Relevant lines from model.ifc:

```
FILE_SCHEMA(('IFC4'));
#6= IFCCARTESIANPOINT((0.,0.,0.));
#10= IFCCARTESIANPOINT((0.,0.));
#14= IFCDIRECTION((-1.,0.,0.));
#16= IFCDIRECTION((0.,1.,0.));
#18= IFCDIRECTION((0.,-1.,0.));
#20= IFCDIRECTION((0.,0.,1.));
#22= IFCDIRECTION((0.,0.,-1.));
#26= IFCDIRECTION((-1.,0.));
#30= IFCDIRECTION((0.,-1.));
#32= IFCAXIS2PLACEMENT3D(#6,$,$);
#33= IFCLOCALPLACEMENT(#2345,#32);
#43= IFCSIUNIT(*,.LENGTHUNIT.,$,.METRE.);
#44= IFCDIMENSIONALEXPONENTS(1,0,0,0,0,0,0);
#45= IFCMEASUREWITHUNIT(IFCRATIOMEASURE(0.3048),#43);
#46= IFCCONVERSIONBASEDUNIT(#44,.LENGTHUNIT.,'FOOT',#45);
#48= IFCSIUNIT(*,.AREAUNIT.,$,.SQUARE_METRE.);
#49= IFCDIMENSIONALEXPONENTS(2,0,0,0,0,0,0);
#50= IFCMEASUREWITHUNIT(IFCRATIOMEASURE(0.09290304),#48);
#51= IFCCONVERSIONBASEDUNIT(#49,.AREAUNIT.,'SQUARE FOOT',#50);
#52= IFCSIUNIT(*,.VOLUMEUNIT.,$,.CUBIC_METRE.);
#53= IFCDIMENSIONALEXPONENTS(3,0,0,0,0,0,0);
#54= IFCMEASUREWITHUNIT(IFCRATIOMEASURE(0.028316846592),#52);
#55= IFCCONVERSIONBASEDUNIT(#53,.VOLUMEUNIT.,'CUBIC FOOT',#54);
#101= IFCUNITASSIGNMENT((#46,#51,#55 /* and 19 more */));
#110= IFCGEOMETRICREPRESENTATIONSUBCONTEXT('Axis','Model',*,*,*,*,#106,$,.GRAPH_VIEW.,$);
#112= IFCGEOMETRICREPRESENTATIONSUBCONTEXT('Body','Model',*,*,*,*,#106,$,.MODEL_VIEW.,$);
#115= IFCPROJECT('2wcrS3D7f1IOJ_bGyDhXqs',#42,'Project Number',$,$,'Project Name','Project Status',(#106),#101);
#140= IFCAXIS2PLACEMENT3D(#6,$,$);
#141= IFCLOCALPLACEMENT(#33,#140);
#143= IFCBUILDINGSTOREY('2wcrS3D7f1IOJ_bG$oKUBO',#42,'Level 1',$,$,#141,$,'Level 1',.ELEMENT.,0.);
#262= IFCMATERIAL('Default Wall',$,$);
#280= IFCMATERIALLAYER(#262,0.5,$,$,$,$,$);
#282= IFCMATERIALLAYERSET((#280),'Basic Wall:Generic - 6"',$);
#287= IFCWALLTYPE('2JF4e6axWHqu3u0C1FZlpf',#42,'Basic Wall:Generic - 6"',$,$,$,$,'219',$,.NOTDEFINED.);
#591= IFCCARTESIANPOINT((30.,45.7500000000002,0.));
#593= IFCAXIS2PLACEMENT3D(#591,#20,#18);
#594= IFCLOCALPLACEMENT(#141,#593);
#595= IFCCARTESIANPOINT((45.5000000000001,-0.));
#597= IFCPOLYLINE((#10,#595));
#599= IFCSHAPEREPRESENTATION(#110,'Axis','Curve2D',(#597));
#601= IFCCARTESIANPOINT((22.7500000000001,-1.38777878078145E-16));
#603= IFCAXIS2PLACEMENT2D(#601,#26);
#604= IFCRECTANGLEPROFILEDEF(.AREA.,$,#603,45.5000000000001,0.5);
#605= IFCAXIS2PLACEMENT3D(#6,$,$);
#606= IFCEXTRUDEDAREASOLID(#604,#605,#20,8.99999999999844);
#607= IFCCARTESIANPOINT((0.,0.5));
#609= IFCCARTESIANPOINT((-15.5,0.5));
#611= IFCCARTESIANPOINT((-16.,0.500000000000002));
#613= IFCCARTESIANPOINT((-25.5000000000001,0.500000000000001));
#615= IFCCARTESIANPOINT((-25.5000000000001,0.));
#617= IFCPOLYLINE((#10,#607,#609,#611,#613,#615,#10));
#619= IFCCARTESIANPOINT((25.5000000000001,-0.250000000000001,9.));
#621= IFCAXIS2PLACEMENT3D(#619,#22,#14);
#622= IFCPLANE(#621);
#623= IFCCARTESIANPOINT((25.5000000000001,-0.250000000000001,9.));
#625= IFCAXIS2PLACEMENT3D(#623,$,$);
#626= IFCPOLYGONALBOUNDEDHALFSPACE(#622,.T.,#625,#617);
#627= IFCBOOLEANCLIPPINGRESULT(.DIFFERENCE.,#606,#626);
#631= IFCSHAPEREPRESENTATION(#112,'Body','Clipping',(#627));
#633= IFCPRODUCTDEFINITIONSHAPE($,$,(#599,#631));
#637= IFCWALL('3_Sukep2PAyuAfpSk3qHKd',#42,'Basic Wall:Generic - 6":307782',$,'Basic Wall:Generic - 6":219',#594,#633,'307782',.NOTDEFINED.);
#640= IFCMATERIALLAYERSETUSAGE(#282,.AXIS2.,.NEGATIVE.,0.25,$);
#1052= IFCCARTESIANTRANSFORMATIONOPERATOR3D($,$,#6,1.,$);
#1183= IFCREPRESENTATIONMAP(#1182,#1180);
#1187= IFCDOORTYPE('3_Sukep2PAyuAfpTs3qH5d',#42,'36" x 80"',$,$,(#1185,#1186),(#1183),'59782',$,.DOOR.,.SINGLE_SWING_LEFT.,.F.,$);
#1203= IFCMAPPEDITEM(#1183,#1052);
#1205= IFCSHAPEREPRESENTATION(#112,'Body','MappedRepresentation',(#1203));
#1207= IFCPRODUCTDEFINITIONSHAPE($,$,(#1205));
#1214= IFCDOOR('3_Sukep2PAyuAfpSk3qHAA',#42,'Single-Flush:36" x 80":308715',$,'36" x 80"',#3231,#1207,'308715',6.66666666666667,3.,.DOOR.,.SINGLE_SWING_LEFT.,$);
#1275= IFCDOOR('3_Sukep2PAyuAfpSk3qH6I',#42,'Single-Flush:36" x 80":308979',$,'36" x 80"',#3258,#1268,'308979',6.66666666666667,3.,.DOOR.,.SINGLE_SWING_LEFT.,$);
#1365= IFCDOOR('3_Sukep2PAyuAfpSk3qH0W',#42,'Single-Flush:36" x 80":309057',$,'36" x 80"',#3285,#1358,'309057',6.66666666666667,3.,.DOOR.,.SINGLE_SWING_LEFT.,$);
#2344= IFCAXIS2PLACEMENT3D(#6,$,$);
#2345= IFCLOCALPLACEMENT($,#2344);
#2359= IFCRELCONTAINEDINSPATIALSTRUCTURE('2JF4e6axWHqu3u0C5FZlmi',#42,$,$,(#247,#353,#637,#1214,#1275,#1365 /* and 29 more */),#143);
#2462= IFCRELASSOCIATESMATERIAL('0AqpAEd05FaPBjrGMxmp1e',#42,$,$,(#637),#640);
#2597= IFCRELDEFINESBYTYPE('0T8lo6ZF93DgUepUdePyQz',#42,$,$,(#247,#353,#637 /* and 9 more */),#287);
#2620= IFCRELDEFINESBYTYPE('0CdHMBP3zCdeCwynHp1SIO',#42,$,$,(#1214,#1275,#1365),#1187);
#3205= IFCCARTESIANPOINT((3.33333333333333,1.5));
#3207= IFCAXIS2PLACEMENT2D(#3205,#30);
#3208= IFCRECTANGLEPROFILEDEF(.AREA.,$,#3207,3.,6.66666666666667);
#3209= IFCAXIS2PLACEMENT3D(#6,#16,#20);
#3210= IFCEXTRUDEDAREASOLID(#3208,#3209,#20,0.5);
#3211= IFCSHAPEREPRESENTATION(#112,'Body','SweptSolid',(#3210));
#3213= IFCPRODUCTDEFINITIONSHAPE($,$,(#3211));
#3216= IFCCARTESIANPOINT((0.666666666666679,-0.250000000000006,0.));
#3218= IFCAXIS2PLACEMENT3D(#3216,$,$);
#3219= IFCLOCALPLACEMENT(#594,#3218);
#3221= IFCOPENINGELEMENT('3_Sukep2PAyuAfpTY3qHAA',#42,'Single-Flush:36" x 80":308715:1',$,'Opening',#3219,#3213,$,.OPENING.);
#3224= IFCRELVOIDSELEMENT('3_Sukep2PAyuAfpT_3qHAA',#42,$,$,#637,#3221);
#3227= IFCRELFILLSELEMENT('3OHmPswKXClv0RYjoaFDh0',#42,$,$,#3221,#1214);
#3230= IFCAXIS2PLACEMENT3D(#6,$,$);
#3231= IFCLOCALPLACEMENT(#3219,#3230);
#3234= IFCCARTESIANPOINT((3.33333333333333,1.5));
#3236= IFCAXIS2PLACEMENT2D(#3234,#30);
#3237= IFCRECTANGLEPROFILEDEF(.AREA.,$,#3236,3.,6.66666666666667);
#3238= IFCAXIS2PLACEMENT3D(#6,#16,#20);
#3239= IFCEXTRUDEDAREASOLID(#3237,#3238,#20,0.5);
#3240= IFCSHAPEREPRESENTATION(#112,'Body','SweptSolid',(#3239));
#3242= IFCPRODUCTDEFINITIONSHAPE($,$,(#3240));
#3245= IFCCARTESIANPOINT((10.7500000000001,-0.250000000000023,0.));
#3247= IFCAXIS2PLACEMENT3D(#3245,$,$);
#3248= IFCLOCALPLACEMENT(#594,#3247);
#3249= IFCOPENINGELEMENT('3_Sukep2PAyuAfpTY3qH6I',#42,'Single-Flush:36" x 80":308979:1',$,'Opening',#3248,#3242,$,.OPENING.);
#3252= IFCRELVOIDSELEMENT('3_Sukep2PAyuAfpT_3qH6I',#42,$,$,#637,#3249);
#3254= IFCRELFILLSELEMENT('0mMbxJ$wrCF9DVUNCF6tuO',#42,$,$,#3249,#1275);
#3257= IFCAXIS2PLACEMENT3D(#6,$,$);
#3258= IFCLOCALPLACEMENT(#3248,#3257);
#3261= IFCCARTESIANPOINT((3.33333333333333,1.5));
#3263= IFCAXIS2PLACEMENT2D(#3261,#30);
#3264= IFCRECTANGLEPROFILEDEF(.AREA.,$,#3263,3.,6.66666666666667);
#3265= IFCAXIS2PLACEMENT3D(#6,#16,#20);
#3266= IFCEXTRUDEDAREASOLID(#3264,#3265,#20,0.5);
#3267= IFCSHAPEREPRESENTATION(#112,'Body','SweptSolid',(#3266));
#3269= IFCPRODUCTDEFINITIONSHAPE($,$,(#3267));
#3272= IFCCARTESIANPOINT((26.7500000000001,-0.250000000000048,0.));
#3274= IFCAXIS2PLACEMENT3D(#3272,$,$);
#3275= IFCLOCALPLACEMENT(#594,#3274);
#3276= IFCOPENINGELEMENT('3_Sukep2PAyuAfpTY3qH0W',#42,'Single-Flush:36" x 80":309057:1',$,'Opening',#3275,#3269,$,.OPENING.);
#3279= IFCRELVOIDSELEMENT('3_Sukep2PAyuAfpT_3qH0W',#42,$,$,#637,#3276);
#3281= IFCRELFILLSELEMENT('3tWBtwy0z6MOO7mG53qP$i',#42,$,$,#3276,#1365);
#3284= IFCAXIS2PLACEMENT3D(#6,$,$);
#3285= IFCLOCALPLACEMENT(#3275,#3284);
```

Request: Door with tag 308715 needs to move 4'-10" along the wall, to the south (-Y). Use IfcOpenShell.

```python
import ifcopenshell
import ifcopenshell.api.geometry
import ifcopenshell.util.placement
import ifcopenshell.util.unit

model = ifcopenshell.open("model.ifc")
unit_scale = ifcopenshell.util.unit.calculate_unit_scale(model)

door = model.by_guid("3_Sukep2PAyuAfpSk3qHAA")
opening = door.FillsVoids[0].RelatingOpeningElement
wall = opening.VoidsElements[0].RelatingBuildingElement

wall_matrix = ifcopenshell.util.placement.get_local_placement(wall.ObjectPlacement)
shift = wall_matrix[:3, 0] * 58 * 0.0254 / unit_scale
before = ifcopenshell.util.placement.get_local_placement(door.ObjectPlacement)[:3, 3].copy()

# The door is placed relative to its opening, so it follows when the opening moves.
matrix = ifcopenshell.util.placement.get_local_placement(opening.ObjectPlacement)
matrix[:3, 3] += shift
ifcopenshell.api.geometry.edit_object_placement(
    model, product=opening, matrix=matrix, is_si=False, should_transform_children=True
)

after = ifcopenshell.util.placement.get_local_placement(door.ObjectPlacement)[:3, 3]
print("door moved by", (after - before).round(3) + 0.0)

model.write("model_v2.ifc")
```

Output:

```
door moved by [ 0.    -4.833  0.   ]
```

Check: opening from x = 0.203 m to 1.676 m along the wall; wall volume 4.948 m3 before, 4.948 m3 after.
